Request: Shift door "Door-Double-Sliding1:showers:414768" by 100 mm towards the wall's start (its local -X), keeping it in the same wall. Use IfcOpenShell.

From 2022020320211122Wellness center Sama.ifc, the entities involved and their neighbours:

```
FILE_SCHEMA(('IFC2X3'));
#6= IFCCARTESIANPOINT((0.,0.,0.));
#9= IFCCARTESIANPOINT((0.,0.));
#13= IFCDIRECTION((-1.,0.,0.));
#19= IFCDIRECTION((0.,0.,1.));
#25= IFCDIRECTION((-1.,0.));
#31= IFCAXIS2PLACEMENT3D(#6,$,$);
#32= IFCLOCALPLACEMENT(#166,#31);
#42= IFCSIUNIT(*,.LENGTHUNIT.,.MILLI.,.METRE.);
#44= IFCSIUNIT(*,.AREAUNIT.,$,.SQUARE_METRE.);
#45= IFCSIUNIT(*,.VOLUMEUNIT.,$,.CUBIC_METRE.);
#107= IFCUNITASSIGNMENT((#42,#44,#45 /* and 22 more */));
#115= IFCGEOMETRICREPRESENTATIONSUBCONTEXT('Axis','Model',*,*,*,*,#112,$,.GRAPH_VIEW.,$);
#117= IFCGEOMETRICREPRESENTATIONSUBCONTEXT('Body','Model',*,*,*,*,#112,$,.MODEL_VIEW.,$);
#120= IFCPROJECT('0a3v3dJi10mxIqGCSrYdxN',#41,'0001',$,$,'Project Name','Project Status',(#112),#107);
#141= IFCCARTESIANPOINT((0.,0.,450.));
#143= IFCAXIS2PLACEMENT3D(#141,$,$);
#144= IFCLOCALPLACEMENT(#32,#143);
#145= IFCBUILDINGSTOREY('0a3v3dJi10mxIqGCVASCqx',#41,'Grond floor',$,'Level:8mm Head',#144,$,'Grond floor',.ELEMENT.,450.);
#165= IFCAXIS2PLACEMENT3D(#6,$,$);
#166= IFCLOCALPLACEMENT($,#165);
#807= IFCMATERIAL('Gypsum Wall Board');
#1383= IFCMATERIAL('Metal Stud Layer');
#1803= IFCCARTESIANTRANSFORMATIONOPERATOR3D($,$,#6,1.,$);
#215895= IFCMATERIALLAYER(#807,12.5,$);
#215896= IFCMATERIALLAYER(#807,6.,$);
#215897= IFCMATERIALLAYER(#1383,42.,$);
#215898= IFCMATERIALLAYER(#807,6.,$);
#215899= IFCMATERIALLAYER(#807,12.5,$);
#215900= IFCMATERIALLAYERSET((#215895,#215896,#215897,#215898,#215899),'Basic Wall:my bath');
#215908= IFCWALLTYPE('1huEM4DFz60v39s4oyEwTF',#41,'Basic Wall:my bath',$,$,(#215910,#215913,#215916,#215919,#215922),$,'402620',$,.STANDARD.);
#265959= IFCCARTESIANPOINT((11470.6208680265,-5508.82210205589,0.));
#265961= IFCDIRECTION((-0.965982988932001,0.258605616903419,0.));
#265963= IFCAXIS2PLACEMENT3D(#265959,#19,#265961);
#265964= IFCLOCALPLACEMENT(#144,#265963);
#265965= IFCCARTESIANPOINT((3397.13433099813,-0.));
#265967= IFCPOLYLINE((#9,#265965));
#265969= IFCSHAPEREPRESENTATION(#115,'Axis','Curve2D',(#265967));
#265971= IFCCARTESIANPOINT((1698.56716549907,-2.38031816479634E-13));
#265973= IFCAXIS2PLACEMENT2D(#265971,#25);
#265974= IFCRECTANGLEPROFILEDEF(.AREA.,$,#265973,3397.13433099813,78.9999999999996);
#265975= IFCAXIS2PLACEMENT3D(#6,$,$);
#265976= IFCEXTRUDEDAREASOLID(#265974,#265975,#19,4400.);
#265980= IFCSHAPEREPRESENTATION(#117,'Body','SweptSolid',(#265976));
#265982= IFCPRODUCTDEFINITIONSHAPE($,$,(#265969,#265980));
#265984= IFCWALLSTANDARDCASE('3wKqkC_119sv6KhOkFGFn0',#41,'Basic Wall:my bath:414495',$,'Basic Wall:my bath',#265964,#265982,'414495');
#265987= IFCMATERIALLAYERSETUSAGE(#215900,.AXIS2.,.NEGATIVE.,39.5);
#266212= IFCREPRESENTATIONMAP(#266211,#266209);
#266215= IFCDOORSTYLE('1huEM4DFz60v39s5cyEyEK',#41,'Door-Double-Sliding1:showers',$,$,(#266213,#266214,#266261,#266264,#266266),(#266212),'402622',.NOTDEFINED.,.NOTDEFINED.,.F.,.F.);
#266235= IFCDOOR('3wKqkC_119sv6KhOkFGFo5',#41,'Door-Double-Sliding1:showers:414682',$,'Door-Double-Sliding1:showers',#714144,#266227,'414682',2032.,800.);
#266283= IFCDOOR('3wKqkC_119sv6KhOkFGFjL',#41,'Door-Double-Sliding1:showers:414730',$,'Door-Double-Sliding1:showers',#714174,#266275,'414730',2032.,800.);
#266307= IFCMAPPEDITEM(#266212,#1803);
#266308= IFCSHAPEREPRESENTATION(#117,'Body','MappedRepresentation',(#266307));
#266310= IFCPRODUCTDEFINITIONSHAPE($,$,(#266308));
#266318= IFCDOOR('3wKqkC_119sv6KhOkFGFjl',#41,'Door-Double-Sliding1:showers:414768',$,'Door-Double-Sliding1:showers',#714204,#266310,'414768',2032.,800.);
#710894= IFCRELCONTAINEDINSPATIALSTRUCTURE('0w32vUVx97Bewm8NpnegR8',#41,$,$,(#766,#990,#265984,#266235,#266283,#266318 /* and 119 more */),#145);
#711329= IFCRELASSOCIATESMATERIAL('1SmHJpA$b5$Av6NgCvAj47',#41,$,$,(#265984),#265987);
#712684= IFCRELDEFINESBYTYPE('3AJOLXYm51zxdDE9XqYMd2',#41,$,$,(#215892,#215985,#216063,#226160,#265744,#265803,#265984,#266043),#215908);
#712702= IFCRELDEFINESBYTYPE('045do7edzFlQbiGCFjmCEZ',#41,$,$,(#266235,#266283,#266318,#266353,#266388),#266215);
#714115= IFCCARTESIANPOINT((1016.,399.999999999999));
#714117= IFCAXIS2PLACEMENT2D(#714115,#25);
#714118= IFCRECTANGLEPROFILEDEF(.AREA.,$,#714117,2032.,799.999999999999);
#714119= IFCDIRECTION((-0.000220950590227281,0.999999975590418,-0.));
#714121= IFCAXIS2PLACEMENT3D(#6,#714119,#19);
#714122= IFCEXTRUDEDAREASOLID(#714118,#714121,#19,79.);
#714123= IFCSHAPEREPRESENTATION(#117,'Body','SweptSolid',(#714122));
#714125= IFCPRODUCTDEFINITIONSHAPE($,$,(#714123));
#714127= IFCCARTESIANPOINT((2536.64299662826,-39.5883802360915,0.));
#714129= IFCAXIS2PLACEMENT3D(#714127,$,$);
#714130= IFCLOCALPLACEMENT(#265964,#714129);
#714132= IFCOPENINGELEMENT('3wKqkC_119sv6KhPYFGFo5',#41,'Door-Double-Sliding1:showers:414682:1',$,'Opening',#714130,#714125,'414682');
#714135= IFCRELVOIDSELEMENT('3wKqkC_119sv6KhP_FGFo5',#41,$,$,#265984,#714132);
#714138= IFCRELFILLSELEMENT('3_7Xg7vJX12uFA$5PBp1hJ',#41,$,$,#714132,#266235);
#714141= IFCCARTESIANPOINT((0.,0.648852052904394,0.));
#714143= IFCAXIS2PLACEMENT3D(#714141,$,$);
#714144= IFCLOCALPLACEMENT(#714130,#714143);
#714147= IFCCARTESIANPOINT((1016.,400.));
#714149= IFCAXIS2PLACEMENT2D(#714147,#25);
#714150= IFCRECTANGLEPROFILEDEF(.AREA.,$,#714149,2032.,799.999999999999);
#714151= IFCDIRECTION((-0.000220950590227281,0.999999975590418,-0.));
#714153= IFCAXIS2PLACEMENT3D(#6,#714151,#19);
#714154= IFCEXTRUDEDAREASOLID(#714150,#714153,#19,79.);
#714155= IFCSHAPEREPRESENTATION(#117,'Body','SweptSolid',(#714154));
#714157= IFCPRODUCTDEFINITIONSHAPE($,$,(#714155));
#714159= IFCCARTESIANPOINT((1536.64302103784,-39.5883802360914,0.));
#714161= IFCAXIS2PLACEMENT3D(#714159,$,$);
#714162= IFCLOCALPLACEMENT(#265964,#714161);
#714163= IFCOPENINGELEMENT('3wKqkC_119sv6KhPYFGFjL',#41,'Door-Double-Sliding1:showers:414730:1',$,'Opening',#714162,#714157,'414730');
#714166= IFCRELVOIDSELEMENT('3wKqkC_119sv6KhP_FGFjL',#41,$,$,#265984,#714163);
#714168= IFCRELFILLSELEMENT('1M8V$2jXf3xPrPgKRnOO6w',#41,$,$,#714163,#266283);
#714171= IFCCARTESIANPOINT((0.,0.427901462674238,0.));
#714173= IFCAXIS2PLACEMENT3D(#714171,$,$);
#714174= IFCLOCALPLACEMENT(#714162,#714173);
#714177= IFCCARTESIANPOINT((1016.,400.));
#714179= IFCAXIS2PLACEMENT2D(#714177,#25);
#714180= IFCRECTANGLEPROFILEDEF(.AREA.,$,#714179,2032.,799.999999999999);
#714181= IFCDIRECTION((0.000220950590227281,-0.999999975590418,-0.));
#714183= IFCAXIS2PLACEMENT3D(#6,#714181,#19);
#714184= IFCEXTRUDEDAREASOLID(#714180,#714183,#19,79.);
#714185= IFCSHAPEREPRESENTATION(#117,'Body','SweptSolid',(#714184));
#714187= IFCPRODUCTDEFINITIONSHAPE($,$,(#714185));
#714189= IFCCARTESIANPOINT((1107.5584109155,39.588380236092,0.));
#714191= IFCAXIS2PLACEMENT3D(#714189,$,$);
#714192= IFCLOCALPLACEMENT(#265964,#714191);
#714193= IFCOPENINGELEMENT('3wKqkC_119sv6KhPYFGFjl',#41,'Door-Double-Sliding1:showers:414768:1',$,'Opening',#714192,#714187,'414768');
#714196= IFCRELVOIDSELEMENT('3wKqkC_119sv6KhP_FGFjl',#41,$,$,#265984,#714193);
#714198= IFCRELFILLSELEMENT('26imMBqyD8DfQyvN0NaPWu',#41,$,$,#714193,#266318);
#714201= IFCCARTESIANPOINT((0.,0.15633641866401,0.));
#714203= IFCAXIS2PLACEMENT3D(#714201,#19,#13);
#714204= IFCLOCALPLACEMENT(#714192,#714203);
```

```python
import ifcopenshell
import ifcopenshell.api.geometry
import ifcopenshell.util.placement
import ifcopenshell.util.unit

model = ifcopenshell.open("2022020320211122Wellness center Sama.ifc")
unit_scale = ifcopenshell.util.unit.calculate_unit_scale(model)

door = model.by_id(266318)
opening = door.FillsVoids[0].RelatingOpeningElement
wall = opening.VoidsElements[0].RelatingBuildingElement

wall_matrix = ifcopenshell.util.placement.get_local_placement(wall.ObjectPlacement)
shift = wall_matrix[:3, 0] * -0.1 / unit_scale
before = ifcopenshell.util.placement.get_local_placement(door.ObjectPlacement)[:3, 3].copy()

# The door is placed relative to its opening, so it follows when the opening moves.
matrix = ifcopenshell.util.placement.get_local_placement(opening.ObjectPlacement)
matrix[:3, 3] += shift
ifcopenshell.api.geometry.edit_object_placement(
    model, product=opening, matrix=matrix, is_si=False, should_transform_children=True
)

after = ifcopenshell.util.placement.get_local_placement(door.ObjectPlacement)[:3, 3]
print("door moved by", (after - before).round(3) + 0.0)

model.write("2022020320211122Wellness center Sama_updated.ifc")
```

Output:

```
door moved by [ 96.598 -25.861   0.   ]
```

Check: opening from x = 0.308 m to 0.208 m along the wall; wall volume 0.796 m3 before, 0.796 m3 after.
